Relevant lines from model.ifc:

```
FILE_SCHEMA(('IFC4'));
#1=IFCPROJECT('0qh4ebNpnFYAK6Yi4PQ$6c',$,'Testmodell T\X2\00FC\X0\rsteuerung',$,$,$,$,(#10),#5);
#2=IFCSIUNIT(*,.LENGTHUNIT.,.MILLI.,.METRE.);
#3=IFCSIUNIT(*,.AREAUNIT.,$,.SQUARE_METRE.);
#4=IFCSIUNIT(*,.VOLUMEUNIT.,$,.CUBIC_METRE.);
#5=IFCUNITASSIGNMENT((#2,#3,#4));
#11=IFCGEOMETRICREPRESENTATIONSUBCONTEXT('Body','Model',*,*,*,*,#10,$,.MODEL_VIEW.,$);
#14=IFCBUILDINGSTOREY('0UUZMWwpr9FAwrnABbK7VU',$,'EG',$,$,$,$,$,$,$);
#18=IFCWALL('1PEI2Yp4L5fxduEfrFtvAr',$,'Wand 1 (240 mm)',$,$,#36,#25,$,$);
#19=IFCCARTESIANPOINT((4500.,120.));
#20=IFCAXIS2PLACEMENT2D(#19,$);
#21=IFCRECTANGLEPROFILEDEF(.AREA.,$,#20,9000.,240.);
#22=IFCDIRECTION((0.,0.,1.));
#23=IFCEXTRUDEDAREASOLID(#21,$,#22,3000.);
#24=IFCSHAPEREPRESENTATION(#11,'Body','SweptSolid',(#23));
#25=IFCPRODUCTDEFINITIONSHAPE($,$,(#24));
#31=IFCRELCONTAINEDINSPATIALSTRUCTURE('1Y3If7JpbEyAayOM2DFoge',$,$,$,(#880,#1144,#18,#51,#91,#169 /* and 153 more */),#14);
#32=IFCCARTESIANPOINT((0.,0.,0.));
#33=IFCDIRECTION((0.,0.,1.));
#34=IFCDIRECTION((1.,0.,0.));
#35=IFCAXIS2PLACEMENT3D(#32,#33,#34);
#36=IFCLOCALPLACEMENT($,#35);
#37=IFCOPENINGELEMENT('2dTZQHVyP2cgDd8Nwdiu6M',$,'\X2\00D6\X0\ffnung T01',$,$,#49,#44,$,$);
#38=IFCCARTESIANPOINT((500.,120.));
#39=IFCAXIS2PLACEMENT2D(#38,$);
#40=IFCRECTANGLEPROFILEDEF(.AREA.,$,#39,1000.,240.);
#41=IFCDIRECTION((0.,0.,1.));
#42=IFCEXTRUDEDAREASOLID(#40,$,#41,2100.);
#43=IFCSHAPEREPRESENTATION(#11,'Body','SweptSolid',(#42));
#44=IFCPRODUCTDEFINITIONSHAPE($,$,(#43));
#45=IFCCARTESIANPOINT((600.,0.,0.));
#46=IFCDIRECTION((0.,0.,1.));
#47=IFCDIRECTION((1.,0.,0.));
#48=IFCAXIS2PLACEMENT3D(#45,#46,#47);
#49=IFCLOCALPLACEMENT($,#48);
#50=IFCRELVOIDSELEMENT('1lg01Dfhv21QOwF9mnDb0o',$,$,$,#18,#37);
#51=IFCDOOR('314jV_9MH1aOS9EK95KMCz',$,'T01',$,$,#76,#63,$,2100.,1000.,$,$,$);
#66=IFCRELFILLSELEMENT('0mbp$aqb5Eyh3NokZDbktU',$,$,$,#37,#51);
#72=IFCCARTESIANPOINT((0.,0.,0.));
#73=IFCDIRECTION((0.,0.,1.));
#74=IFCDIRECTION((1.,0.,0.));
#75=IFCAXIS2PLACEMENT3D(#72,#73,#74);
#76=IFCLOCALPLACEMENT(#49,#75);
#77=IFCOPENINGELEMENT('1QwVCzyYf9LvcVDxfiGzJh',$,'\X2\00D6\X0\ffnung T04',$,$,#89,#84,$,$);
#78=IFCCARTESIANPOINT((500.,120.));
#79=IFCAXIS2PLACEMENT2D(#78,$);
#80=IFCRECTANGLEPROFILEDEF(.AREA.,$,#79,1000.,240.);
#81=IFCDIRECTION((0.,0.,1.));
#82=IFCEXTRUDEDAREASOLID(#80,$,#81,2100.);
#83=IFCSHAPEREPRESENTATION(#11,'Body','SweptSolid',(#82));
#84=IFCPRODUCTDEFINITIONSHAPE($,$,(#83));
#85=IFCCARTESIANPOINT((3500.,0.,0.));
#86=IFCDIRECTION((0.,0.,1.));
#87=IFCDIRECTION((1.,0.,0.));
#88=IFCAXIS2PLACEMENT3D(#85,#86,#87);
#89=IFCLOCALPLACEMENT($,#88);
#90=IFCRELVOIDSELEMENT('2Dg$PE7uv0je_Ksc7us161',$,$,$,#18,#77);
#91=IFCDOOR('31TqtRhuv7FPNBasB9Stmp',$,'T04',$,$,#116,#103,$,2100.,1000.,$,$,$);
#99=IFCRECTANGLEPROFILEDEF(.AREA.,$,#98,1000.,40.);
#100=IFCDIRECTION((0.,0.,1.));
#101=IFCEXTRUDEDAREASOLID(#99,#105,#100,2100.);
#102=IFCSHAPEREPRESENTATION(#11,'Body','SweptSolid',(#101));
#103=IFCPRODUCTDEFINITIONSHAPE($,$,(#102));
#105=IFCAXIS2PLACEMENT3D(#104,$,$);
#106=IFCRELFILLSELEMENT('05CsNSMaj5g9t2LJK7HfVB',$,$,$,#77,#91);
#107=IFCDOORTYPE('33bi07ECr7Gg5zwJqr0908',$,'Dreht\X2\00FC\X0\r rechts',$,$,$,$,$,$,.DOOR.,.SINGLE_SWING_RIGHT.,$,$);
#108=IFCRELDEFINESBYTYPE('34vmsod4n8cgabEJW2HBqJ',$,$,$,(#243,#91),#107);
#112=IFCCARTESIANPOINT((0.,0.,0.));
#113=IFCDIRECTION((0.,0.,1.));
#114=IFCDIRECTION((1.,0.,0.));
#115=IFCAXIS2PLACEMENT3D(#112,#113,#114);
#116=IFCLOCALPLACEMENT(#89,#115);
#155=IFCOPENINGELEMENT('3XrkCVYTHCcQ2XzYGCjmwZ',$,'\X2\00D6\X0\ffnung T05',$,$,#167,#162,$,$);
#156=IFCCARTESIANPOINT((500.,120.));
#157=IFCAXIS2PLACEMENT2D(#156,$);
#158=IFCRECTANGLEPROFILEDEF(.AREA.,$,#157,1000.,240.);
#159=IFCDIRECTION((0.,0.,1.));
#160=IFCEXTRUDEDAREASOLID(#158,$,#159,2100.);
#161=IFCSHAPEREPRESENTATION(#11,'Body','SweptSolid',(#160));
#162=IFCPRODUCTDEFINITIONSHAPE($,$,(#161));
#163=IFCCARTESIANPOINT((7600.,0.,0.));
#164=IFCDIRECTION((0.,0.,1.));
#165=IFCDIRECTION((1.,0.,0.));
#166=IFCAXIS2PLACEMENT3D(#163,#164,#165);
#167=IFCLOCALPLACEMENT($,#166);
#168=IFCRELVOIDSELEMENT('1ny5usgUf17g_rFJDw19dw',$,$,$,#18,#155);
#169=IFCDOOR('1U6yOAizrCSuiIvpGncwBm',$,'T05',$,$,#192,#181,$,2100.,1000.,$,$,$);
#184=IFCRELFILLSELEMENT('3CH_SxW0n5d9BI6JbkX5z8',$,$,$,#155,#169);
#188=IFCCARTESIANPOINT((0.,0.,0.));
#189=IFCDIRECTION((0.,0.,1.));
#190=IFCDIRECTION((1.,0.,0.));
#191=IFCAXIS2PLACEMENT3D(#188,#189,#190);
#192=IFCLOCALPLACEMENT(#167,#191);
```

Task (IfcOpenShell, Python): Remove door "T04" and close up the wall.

```python
import ifcopenshell
import ifcopenshell.api.feature
import ifcopenshell.api.root
import ifcopenshell.geom
import ifcopenshell.util.shape

model = ifcopenshell.open("model.ifc")
settings = ifcopenshell.geom.settings()


def volume(element):
    """Net volume in cubic metres, openings subtracted."""
    shape = ifcopenshell.geom.create_shape(settings, element)
    return ifcopenshell.util.shape.get_volume(shape.geometry)


door = model.by_guid("31TqtRhuv7FPNBasB9Stmp")
opening = door.FillsVoids[0].RelatingOpeningElement
wall = opening.VoidsElements[0].RelatingBuildingElement
before = volume(wall)

ifcopenshell.api.root.remove_product(model, product=door)
ifcopenshell.api.feature.remove_feature(model, feature=opening)

after = volume(wall)

print(f"wall volume {before:.3f} -> {after:.3f} m3")

model.write("model-out.ifc")
```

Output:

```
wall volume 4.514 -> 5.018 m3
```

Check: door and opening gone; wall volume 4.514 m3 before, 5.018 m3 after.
